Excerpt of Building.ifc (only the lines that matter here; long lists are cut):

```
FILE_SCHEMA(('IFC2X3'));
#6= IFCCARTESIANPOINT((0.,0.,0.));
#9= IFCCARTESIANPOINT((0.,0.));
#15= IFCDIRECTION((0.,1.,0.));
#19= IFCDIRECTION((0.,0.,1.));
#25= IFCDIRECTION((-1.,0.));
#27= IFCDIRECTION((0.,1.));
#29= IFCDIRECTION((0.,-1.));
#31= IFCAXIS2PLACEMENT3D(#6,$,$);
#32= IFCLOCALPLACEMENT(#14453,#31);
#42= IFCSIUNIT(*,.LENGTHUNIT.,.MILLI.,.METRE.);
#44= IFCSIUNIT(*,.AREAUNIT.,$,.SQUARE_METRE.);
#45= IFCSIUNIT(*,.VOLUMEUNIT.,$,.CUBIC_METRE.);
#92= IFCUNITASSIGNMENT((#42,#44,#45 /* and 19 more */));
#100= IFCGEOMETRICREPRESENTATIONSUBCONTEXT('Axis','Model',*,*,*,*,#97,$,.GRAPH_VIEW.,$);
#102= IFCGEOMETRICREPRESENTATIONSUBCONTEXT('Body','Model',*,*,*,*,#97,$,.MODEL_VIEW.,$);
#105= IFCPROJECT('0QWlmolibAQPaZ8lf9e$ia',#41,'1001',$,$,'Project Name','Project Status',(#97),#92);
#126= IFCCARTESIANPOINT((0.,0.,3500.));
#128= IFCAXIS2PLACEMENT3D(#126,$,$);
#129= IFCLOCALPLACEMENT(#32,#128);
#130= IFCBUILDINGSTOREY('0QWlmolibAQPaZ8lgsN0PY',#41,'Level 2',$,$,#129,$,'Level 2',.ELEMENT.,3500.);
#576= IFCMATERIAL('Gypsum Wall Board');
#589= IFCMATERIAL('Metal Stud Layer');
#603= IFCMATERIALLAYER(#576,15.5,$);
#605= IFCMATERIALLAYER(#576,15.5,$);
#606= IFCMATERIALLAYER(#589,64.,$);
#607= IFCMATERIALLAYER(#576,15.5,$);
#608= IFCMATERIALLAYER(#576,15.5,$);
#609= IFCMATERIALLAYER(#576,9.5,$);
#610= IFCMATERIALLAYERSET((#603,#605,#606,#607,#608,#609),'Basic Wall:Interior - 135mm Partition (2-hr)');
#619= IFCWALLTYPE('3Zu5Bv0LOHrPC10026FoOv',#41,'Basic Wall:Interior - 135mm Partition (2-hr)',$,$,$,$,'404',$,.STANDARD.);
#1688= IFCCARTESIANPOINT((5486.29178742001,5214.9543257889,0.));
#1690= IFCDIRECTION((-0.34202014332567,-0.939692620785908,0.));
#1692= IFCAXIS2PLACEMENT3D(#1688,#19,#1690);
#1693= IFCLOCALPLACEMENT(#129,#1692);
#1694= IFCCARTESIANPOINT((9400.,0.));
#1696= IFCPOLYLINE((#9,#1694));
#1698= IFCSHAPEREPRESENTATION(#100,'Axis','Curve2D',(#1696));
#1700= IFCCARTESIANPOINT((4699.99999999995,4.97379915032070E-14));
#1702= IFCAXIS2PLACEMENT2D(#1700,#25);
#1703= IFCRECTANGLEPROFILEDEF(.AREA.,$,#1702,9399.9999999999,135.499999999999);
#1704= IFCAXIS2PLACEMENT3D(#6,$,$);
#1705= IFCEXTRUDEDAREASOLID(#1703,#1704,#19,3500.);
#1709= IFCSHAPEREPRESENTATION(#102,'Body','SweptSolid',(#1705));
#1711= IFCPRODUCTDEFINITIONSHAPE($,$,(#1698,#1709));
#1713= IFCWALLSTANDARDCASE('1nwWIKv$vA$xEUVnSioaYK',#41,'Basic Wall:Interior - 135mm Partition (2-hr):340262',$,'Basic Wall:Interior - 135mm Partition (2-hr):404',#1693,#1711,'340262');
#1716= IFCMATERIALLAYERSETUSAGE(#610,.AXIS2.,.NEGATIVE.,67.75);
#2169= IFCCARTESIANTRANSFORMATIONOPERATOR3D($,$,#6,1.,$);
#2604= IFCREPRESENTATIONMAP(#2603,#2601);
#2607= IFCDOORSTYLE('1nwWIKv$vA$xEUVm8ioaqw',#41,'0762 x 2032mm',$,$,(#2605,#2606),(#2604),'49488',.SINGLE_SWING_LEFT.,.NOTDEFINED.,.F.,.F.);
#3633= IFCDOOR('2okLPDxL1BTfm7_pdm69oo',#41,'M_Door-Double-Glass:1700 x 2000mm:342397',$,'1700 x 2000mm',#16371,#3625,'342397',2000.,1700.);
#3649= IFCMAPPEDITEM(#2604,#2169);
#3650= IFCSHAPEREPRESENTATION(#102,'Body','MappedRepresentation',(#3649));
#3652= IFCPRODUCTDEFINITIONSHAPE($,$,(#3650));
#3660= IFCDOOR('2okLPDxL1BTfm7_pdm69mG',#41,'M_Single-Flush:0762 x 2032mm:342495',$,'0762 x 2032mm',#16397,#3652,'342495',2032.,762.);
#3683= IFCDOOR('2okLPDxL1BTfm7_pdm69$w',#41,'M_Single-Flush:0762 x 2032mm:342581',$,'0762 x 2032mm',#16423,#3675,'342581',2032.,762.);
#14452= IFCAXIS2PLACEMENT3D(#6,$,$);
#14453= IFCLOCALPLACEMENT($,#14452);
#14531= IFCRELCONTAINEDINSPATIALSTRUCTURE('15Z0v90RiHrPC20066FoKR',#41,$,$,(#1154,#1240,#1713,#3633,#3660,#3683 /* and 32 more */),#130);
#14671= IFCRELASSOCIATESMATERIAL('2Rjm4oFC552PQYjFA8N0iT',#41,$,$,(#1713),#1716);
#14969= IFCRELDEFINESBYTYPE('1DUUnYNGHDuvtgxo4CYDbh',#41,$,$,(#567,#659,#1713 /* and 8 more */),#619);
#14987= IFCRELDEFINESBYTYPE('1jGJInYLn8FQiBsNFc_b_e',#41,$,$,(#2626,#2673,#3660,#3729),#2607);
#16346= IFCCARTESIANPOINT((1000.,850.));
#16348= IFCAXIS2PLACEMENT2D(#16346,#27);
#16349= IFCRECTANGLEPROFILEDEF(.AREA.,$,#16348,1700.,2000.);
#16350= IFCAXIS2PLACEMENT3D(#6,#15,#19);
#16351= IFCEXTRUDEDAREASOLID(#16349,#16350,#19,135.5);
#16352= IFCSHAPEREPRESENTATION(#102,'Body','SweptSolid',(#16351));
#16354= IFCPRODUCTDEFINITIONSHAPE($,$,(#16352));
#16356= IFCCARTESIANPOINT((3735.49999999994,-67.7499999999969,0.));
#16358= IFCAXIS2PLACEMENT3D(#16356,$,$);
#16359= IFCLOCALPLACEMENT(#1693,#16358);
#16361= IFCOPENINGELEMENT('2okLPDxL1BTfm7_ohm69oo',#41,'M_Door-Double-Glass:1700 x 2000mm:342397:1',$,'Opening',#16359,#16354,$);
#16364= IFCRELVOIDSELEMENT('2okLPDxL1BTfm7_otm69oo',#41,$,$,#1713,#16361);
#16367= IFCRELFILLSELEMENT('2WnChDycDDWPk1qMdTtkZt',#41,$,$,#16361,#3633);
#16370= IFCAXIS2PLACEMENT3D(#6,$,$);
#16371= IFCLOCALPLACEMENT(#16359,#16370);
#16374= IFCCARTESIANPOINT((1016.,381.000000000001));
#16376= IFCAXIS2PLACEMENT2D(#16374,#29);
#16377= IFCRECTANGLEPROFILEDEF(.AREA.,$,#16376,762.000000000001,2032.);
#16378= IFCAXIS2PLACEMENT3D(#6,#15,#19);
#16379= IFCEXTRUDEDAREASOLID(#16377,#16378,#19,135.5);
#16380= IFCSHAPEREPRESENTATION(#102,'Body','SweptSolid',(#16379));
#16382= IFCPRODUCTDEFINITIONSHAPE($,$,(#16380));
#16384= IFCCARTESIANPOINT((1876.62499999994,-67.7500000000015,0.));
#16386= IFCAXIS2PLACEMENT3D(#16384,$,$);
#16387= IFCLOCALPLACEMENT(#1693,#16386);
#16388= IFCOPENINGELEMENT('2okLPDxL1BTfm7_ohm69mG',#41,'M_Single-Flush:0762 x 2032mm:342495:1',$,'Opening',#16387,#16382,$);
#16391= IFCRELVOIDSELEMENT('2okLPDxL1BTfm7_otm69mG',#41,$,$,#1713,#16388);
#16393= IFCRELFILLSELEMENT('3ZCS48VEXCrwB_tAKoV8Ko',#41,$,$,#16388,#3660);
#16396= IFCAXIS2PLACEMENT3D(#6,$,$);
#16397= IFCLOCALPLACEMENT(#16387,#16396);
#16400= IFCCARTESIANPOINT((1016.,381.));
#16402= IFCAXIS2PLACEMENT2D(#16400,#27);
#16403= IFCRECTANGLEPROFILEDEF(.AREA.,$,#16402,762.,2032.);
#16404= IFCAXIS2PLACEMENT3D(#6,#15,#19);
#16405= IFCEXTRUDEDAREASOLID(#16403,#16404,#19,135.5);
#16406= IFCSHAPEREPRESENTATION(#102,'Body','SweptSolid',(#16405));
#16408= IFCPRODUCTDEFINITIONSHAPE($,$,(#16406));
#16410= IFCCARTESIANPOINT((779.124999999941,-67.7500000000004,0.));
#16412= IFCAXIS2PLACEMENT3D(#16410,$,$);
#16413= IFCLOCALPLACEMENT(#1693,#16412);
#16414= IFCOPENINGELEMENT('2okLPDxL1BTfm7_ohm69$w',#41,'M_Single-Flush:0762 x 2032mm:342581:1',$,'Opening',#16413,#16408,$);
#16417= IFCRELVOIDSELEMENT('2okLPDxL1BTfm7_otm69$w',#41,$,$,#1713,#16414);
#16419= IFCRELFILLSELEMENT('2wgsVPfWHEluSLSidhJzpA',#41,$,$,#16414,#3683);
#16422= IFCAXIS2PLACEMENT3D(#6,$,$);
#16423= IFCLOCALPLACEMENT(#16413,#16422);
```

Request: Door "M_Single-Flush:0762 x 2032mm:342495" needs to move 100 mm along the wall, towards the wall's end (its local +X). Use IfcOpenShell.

```python
import ifcopenshell
import ifcopenshell.api.geometry
import ifcopenshell.util.placement

model = ifcopenshell.open("Building.ifc")

door = model.by_id(3660)
opening = door.FillsVoids[0].RelatingOpeningElement
wall = opening.VoidsElements[0].RelatingBuildingElement

wall_matrix = ifcopenshell.util.placement.get_local_placement(wall.ObjectPlacement)
shift = wall_matrix[:3, 0] * 100.0
before = ifcopenshell.util.placement.get_local_placement(door.ObjectPlacement)[:3, 3].copy()

# The door is placed relative to its opening, so it follows when the opening moves.
matrix = ifcopenshell.util.placement.get_local_placement(opening.ObjectPlacement)
matrix[:3, 3] += shift
ifcopenshell.api.geometry.edit_object_placement(
    model, product=opening, matrix=matrix, is_si=False, should_transform_children=True
)

after = ifcopenshell.util.placement.get_local_placement(door.ObjectPlacement)[:3, 3]
print("door moved by", (after - before).round(3) + 0.0)

model.write("Building_updated.ifc")
```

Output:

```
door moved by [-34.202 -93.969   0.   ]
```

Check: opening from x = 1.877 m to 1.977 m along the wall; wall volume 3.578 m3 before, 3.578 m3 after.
